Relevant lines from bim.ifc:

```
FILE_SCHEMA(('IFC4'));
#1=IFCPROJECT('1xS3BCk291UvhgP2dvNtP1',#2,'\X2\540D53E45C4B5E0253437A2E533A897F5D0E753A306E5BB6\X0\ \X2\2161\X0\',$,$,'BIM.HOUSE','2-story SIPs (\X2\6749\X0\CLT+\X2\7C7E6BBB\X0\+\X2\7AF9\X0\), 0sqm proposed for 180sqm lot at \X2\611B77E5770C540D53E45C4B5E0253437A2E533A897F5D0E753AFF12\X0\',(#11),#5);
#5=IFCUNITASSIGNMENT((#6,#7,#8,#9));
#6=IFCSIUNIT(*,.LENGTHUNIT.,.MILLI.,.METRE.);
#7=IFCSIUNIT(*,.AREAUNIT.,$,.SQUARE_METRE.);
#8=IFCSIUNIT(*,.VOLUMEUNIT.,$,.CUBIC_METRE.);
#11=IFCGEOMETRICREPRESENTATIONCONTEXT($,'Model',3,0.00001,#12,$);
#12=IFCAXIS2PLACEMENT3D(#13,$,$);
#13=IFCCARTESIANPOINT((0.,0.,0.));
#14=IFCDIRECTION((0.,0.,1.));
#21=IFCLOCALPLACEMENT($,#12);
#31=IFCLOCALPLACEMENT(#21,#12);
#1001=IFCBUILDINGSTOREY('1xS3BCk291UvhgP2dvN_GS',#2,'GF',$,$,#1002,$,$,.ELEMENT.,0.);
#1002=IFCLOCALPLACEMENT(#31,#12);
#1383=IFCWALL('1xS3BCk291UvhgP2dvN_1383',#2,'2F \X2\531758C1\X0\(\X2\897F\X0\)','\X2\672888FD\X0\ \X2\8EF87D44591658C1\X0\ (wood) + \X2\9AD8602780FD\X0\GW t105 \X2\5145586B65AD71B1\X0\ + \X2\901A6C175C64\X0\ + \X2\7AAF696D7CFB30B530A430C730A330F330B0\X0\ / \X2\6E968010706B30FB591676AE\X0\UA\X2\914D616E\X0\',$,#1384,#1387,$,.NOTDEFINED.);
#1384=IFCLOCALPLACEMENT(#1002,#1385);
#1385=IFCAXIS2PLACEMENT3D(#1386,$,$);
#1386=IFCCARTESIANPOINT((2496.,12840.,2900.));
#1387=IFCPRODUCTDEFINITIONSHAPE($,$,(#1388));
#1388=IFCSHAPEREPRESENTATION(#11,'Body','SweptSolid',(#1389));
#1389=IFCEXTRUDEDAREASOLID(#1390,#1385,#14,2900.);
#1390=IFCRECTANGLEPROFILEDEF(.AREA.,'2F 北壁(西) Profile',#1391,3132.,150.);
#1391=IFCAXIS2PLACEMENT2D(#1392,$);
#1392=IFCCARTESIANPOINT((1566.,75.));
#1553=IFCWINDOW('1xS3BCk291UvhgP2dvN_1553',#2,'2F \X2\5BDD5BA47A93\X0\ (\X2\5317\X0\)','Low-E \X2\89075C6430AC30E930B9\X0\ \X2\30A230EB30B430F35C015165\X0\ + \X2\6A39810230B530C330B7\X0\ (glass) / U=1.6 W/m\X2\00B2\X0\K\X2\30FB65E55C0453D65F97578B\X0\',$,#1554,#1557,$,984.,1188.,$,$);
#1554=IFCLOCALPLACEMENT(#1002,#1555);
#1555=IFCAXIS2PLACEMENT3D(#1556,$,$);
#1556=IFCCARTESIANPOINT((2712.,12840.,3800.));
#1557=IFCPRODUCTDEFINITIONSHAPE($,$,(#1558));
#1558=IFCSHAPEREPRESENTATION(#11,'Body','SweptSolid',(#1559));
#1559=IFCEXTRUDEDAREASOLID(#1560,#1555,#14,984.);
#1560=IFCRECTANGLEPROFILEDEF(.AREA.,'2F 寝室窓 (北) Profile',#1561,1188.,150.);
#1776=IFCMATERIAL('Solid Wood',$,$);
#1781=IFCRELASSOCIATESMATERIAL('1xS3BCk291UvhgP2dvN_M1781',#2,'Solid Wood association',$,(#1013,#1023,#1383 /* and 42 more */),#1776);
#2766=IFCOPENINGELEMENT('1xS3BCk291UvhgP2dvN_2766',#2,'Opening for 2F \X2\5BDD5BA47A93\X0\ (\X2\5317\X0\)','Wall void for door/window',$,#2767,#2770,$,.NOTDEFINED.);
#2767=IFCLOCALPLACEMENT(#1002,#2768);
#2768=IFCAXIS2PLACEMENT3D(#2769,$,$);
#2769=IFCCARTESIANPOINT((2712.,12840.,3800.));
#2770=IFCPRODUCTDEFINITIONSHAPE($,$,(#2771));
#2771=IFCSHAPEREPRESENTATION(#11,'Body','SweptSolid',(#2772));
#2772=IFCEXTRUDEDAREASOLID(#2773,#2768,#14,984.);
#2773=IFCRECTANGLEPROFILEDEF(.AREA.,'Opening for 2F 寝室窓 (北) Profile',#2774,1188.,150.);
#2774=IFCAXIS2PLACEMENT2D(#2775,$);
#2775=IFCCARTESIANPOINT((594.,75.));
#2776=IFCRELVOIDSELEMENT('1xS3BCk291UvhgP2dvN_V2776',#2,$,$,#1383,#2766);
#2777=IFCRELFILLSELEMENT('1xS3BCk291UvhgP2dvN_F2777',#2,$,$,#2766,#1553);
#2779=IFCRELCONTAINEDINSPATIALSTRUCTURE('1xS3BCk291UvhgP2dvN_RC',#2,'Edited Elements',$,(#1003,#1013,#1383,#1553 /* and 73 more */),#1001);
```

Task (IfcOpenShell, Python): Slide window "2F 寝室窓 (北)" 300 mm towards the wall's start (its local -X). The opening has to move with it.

```python
import ifcopenshell
import ifcopenshell.api.geometry
import ifcopenshell.util.placement
import ifcopenshell.util.unit

model = ifcopenshell.open("bim.ifc")
unit_scale = ifcopenshell.util.unit.calculate_unit_scale(model)

window = model.by_guid("1xS3BCk291UvhgP2dvN_1553")
opening = window.FillsVoids[0].RelatingOpeningElement
wall = opening.VoidsElements[0].RelatingBuildingElement

wall_matrix = ifcopenshell.util.placement.get_local_placement(wall.ObjectPlacement)
shift = wall_matrix[:3, 0] * -0.3 / unit_scale
before = ifcopenshell.util.placement.get_local_placement(window.ObjectPlacement)[:3, 3].copy()

# The window is not placed relative to its opening, so move both.
for product in (opening, window):
    matrix = ifcopenshell.util.placement.get_local_placement(product.ObjectPlacement)
    matrix[:3, 3] += shift
    ifcopenshell.api.geometry.edit_object_placement(model, product=product, matrix=matrix, is_si=False)

after = ifcopenshell.util.placement.get_local_placement(window.ObjectPlacement)[:3, 3]
print("window moved by", (after - before).round(3) + 0.0)

model.write("bim_edited.ifc")
```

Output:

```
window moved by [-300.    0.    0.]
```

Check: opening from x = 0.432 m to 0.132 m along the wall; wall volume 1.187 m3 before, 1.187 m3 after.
